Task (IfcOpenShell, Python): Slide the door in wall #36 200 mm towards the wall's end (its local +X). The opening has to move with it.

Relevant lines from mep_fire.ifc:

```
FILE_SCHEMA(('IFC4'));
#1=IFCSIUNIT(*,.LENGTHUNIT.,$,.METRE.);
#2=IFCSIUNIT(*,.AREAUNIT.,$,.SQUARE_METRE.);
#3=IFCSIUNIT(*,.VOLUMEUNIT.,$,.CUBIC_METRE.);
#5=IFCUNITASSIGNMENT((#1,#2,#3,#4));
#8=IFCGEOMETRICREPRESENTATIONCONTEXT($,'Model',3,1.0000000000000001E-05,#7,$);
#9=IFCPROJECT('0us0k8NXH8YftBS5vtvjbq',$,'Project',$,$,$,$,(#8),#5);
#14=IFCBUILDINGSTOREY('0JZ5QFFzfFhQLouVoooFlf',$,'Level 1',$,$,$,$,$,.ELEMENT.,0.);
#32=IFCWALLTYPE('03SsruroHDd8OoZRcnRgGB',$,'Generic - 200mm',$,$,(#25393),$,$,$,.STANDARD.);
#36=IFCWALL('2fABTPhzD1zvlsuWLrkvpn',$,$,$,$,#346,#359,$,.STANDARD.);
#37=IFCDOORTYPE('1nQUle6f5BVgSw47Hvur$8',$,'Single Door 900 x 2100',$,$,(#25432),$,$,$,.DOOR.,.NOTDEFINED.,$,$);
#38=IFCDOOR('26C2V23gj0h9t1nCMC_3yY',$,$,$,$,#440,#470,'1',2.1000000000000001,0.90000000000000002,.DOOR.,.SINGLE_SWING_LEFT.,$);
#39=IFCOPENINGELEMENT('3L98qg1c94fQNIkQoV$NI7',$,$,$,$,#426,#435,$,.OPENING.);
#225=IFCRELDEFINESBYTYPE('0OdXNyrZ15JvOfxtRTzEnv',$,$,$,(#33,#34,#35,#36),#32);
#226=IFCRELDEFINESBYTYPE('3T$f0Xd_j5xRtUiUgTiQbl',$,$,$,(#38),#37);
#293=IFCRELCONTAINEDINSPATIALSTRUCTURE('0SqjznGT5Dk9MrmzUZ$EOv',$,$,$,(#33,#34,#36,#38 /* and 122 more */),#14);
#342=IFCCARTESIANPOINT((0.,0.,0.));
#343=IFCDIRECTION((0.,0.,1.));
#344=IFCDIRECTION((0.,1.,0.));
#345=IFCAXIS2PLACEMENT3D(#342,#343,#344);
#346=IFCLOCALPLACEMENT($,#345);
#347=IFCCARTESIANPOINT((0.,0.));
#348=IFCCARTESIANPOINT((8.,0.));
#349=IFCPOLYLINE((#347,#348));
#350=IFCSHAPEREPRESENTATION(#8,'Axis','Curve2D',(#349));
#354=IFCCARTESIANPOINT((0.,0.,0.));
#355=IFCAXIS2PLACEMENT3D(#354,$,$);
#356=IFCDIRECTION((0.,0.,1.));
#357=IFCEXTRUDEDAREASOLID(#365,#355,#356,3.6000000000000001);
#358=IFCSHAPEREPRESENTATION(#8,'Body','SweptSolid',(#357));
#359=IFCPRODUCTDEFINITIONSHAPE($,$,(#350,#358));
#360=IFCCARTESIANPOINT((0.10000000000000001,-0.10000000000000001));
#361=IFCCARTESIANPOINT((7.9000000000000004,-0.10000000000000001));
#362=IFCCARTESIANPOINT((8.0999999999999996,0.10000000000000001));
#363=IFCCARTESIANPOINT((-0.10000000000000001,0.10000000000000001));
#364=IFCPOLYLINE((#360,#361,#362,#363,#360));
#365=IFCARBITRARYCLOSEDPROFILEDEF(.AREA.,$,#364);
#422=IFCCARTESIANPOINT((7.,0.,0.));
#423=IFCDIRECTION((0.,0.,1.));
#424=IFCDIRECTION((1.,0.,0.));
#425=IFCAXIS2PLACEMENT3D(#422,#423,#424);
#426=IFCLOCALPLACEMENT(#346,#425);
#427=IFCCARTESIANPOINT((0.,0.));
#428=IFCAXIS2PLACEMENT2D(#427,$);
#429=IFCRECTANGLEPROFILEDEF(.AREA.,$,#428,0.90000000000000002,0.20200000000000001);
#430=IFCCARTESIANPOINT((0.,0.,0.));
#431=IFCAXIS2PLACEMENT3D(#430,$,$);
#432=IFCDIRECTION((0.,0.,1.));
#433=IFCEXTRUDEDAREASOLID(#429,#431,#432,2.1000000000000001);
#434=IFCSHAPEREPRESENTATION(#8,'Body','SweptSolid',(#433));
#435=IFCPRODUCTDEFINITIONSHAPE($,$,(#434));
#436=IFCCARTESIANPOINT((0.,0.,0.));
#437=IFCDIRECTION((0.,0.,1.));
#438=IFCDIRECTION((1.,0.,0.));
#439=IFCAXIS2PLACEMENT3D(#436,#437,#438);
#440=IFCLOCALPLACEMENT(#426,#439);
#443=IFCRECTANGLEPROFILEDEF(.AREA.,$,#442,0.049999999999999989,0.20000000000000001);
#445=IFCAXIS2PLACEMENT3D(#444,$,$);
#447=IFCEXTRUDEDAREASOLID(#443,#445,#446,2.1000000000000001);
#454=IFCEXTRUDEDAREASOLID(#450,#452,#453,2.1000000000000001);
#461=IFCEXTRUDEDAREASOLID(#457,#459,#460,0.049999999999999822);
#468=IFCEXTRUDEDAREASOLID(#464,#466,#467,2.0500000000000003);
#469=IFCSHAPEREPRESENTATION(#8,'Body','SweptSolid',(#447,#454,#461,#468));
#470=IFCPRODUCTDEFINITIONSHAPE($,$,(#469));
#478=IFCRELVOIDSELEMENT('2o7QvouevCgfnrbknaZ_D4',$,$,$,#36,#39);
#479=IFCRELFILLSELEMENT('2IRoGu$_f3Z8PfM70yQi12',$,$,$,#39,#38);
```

```python
import ifcopenshell
import ifcopenshell.api.geometry
import ifcopenshell.util.placement
import ifcopenshell.util.unit

model = ifcopenshell.open("mep_fire.ifc")
unit_scale = ifcopenshell.util.unit.calculate_unit_scale(model)

door = model.by_guid("26C2V23gj0h9t1nCMC_3yY")
opening = door.FillsVoids[0].RelatingOpeningElement
wall = opening.VoidsElements[0].RelatingBuildingElement

wall_matrix = ifcopenshell.util.placement.get_local_placement(wall.ObjectPlacement)
shift = wall_matrix[:3, 0] * 0.2 / unit_scale
before = ifcopenshell.util.placement.get_local_placement(door.ObjectPlacement)[:3, 3].copy()

# The door is placed relative to its opening, so it follows when the opening moves.
matrix = ifcopenshell.util.placement.get_local_placement(opening.ObjectPlacement)
matrix[:3, 3] += shift
ifcopenshell.api.geometry.edit_object_placement(
    model, product=opening, matrix=matrix, is_si=False, should_transform_children=True
)

after = ifcopenshell.util.placement.get_local_placement(door.ObjectPlacement)[:3, 3]
print("door moved by", (after - before).round(3) + 0.0)

model.write("mep_fire_updated.ifc")
```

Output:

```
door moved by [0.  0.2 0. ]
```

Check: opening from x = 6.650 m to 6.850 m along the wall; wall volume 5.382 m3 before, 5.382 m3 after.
